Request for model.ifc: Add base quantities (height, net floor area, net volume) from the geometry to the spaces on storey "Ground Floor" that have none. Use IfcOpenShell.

First a look at what the model holds.

```python
import ifcopenshell
import ifcopenshell.util.element
import ifcopenshell.util.unit

model = ifcopenshell.open("model.ifc")
print(model.schema)
for unit_type in ("LENGTHUNIT", "AREAUNIT", "VOLUMEUNIT"):
    print(unit_type, ifcopenshell.util.unit.calculate_unit_scale(model, unit_type))
storey = next(s for s in model.by_type("IfcBuildingStorey") if s.Name == "Ground Floor")
spaces = [e for e in ifcopenshell.util.element.get_decomposition(storey) if e.is_a("IfcSpace")]
for e in sorted(spaces, key=lambda e: e.id()):
    print(e.id(), e.is_a(), e.Name, list(ifcopenshell.util.element.get_psets(e, qtos_only=True)), sep=" | ")
```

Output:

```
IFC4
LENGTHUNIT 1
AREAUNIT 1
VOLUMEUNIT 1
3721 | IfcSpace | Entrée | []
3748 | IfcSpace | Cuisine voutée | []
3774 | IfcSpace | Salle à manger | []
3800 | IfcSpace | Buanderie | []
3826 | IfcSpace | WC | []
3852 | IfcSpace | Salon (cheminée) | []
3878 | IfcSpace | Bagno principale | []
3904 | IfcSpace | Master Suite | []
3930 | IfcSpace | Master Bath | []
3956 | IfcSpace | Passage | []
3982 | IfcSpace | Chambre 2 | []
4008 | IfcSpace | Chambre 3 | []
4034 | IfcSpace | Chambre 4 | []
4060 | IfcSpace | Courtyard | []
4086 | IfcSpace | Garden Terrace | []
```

```python
import ifcopenshell
import ifcopenshell.api.pset
import ifcopenshell.geom
import ifcopenshell.util.element
import ifcopenshell.util.shape
import ifcopenshell.util.unit

model = ifcopenshell.open("model.ifc")
unit_scale = ifcopenshell.util.unit.calculate_unit_scale(model)
area_scale = ifcopenshell.util.unit.calculate_unit_scale(model, "AREAUNIT")
volume_scale = ifcopenshell.util.unit.calculate_unit_scale(model, "VOLUMEUNIT")
settings = ifcopenshell.geom.settings()

storey = next(s for s in model.by_type("IfcBuildingStorey") if s.Name == "Ground Floor")
spaces = [e for e in ifcopenshell.util.element.get_decomposition(storey) if e.is_a("IfcSpace")]

for e in sorted(spaces, key=lambda e: e.id()):
    if ifcopenshell.util.element.get_psets(e, qtos_only=True, should_inherit=False):
        continue
    # Geometry comes back in metres, in the element's own axes.
    shape = ifcopenshell.geom.create_shape(settings, e)
    values = {
        "Height": ifcopenshell.util.shape.get_z(shape.geometry) / unit_scale,
        "NetFloorArea": ifcopenshell.util.shape.get_footprint_area(shape.geometry) / area_scale,
        "NetVolume": ifcopenshell.util.shape.get_volume(shape.geometry) / volume_scale,
    }
    qto = ifcopenshell.api.pset.add_qto(model, product=e, name="Qto_SpaceBaseQuantities")
    ifcopenshell.api.pset.edit_qto(model, qto=qto, properties=values)
    print(e.id(), {k: round(v, 3) for k, v in values.items()})

model.write("model-out.ifc")
```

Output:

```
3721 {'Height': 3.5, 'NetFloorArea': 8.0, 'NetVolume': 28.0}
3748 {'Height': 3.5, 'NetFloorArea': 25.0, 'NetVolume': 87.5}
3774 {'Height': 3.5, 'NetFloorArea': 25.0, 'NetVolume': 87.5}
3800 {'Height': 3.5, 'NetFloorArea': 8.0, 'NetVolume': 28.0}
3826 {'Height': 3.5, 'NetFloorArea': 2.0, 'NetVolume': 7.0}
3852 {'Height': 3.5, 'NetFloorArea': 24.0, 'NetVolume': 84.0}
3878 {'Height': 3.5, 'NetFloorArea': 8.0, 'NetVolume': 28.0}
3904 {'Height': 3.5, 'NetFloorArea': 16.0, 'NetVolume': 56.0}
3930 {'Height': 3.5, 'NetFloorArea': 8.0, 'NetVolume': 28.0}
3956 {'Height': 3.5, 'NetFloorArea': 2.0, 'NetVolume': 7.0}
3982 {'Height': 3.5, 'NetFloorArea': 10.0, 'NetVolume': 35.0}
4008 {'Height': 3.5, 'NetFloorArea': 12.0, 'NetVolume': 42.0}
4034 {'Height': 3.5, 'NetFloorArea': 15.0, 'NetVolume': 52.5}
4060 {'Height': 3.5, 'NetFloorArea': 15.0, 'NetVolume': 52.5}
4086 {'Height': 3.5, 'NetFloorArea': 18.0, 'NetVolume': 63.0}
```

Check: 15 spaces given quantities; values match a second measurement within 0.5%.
